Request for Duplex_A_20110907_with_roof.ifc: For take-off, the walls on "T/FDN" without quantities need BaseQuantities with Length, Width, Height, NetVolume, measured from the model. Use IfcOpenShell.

First a look at what the model holds.

```python
import ifcopenshell
import ifcopenshell.util.element
import ifcopenshell.util.unit

model = ifcopenshell.open("Duplex_A_20110907_with_roof.ifc")
print(model.schema)
for unit_type in ("LENGTHUNIT", "AREAUNIT", "VOLUMEUNIT"):
    print(unit_type, ifcopenshell.util.unit.calculate_unit_scale(model, unit_type))
storey = next(s for s in model.by_type("IfcBuildingStorey") if s.Name == "T/FDN")
walls = [e for e in ifcopenshell.util.element.get_decomposition(storey) if e.is_a("IfcWall")]
for e in sorted(walls, key=lambda e: e.id()):
    print(e.id(), e.is_a(), e.Name, list(ifcopenshell.util.element.get_psets(e, qtos_only=True)), sep=" | ")
```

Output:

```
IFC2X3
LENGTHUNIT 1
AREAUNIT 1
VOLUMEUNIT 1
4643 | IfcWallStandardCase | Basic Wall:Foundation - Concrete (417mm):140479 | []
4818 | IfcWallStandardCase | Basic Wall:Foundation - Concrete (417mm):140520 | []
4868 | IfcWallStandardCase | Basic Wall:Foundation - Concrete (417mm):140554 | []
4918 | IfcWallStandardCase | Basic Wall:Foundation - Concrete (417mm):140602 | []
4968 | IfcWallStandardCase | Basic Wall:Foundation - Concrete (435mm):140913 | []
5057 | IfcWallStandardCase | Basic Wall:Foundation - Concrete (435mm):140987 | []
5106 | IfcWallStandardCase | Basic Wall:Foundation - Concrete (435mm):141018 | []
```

```python
import ifcopenshell
import ifcopenshell.api.pset
import ifcopenshell.geom
import ifcopenshell.util.element
import ifcopenshell.util.shape
import ifcopenshell.util.unit

model = ifcopenshell.open("Duplex_A_20110907_with_roof.ifc")
unit_scale = ifcopenshell.util.unit.calculate_unit_scale(model)
volume_scale = ifcopenshell.util.unit.calculate_unit_scale(model, "VOLUMEUNIT")
settings = ifcopenshell.geom.settings()

storey = next(s for s in model.by_type("IfcBuildingStorey") if s.Name == "T/FDN")
walls = [e for e in ifcopenshell.util.element.get_decomposition(storey) if e.is_a("IfcWall")]

for e in sorted(walls, key=lambda e: e.id()):
    if ifcopenshell.util.element.get_psets(e, qtos_only=True, should_inherit=False):
        continue
    # Geometry comes back in metres, in the element's own axes.
    shape = ifcopenshell.geom.create_shape(settings, e)
    values = {
        "Length": ifcopenshell.util.shape.get_x(shape.geometry) / unit_scale,
        "Width": ifcopenshell.util.shape.get_y(shape.geometry) / unit_scale,
        "Height": ifcopenshell.util.shape.get_z(shape.geometry) / unit_scale,
        "NetVolume": ifcopenshell.util.shape.get_volume(shape.geometry) / volume_scale,
    }
    qto = ifcopenshell.api.pset.add_qto(model, product=e, name="BaseQuantities")
    ifcopenshell.api.pset.edit_qto(model, qto=qto, properties=values)
    print(e.id(), {k: round(v, 3) for k, v in values.items()})

model.write("Duplex_A_20110907_with_roof-out.ifc")
```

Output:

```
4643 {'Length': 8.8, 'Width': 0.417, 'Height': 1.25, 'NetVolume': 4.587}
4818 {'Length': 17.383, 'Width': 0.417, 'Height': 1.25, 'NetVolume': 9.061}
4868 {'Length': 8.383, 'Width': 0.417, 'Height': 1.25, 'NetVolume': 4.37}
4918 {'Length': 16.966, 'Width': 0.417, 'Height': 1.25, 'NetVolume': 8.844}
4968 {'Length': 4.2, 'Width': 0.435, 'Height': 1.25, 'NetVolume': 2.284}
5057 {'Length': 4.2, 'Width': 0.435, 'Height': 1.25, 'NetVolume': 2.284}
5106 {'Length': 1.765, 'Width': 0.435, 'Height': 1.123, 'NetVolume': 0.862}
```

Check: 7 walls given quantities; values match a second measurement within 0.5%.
